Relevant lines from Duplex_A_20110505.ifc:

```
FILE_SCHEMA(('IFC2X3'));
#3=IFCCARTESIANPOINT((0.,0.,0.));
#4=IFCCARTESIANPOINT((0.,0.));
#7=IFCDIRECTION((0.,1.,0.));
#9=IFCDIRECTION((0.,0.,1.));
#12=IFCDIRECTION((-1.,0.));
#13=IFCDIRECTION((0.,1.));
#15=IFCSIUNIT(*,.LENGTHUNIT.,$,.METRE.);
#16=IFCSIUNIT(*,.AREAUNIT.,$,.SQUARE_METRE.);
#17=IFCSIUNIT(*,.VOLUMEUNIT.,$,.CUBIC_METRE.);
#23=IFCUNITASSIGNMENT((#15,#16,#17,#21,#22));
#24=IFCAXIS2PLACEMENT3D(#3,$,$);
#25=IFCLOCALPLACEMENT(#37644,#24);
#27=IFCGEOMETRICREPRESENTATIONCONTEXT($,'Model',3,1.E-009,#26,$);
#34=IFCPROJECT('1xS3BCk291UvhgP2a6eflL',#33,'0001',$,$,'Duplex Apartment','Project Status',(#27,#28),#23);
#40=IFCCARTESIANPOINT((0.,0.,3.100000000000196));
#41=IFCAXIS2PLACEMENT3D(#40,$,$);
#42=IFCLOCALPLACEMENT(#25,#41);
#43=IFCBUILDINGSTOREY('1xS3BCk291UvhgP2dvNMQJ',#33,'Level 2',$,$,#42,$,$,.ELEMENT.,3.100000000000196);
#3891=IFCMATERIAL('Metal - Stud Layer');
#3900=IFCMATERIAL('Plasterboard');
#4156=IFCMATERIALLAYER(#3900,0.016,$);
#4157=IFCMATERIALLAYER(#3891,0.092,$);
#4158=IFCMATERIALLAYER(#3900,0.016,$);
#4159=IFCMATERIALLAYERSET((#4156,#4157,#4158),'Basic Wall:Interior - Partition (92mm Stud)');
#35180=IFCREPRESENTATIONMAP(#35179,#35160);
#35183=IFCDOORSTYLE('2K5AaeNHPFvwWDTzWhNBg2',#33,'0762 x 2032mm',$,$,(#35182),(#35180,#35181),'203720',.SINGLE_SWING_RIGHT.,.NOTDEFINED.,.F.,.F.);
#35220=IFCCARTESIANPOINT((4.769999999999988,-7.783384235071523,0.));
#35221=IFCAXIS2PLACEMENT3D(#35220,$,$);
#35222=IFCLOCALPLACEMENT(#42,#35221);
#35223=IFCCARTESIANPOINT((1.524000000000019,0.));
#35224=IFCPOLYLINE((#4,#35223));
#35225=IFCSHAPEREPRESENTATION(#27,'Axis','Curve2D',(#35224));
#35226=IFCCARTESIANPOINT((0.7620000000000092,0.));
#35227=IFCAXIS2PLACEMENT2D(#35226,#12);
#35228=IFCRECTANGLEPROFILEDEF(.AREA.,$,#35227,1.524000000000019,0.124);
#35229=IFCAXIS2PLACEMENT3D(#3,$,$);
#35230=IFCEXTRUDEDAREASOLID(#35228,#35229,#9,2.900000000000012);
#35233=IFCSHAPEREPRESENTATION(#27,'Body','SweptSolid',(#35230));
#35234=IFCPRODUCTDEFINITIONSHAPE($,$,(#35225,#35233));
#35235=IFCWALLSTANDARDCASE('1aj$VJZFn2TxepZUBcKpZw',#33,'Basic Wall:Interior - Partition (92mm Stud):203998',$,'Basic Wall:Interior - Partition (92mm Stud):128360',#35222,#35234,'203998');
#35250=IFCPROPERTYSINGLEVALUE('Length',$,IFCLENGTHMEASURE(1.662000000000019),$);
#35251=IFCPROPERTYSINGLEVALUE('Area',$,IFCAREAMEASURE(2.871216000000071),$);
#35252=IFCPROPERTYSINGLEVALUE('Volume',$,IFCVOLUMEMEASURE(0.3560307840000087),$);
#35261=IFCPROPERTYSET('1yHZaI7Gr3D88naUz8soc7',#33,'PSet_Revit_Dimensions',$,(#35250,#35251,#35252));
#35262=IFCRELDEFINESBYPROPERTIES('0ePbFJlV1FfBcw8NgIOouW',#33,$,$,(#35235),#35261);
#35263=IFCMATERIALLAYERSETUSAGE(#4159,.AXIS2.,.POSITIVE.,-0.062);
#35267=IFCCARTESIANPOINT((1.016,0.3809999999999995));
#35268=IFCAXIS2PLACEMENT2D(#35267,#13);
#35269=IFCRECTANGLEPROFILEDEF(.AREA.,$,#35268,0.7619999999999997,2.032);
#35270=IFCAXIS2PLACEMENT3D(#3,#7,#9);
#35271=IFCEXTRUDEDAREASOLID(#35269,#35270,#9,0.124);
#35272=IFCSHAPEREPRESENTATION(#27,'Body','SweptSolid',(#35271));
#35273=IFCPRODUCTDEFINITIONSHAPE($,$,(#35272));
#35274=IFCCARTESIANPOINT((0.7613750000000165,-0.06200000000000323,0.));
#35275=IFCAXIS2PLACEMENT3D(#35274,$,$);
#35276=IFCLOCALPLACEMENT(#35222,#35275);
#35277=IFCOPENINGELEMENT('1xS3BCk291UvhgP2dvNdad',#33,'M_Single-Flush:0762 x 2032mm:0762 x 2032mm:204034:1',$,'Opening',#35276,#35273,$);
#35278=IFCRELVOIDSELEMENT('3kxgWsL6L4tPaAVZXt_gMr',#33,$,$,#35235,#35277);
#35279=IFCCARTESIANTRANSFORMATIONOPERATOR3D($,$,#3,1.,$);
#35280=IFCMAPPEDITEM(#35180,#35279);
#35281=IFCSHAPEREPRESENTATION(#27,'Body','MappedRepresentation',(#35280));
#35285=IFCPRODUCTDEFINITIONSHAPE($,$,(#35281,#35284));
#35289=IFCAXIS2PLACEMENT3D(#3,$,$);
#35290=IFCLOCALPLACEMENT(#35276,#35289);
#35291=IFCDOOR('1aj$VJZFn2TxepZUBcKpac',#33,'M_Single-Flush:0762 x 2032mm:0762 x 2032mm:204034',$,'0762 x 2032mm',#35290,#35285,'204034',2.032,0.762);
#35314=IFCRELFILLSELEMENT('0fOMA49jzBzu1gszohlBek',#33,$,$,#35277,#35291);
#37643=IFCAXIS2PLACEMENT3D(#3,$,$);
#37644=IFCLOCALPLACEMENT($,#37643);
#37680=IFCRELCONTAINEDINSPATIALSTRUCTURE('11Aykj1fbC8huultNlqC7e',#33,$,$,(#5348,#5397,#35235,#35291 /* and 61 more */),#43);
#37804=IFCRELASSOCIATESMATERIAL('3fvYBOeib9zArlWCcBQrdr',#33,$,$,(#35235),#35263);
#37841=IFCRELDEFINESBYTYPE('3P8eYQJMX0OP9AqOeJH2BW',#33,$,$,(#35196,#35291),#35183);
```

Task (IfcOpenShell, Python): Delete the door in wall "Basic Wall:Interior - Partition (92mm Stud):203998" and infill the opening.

```python
import ifcopenshell
import ifcopenshell.api.feature
import ifcopenshell.api.pset
import ifcopenshell.api.root
import ifcopenshell.geom
import ifcopenshell.util.element
import ifcopenshell.util.shape
import ifcopenshell.util.unit

model = ifcopenshell.open("Duplex_A_20110505.ifc")
area_scale = ifcopenshell.util.unit.calculate_unit_scale(model, "AREAUNIT")
volume_scale = ifcopenshell.util.unit.calculate_unit_scale(model, "VOLUMEUNIT")
settings = ifcopenshell.geom.settings()


def volume(element):
    """Net volume in cubic metres, openings subtracted."""
    shape = ifcopenshell.geom.create_shape(settings, element)
    return ifcopenshell.util.shape.get_volume(shape.geometry)


door = model.by_guid("1aj$VJZFn2TxepZUBcKpac")
opening = door.FillsVoids[0].RelatingOpeningElement
wall = opening.VoidsElements[0].RelatingBuildingElement
before = volume(wall)

ifcopenshell.api.root.remove_product(model, product=door)
ifcopenshell.api.feature.remove_feature(model, feature=opening)

after = volume(wall)
thickness = 0.124  # wall thickness in metres

# Update the wall's stored quantities.
pset = model.by_id(ifcopenshell.util.element.get_pset(wall, "PSet_Revit_Dimensions", should_inherit=False)["id"])
ifcopenshell.api.pset.edit_pset(model, pset=pset, properties={
    "Area": model.create_entity("IfcAreaMeasure", after / thickness / area_scale),
    "Volume": model.create_entity("IfcVolumeMeasure", after / volume_scale),
})

print(f"wall volume {before:.3f} -> {after:.3f} m3")

model.write("Duplex_A_20110505_updated.ifc")
```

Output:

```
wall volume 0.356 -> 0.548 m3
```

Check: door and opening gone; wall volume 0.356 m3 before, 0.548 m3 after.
